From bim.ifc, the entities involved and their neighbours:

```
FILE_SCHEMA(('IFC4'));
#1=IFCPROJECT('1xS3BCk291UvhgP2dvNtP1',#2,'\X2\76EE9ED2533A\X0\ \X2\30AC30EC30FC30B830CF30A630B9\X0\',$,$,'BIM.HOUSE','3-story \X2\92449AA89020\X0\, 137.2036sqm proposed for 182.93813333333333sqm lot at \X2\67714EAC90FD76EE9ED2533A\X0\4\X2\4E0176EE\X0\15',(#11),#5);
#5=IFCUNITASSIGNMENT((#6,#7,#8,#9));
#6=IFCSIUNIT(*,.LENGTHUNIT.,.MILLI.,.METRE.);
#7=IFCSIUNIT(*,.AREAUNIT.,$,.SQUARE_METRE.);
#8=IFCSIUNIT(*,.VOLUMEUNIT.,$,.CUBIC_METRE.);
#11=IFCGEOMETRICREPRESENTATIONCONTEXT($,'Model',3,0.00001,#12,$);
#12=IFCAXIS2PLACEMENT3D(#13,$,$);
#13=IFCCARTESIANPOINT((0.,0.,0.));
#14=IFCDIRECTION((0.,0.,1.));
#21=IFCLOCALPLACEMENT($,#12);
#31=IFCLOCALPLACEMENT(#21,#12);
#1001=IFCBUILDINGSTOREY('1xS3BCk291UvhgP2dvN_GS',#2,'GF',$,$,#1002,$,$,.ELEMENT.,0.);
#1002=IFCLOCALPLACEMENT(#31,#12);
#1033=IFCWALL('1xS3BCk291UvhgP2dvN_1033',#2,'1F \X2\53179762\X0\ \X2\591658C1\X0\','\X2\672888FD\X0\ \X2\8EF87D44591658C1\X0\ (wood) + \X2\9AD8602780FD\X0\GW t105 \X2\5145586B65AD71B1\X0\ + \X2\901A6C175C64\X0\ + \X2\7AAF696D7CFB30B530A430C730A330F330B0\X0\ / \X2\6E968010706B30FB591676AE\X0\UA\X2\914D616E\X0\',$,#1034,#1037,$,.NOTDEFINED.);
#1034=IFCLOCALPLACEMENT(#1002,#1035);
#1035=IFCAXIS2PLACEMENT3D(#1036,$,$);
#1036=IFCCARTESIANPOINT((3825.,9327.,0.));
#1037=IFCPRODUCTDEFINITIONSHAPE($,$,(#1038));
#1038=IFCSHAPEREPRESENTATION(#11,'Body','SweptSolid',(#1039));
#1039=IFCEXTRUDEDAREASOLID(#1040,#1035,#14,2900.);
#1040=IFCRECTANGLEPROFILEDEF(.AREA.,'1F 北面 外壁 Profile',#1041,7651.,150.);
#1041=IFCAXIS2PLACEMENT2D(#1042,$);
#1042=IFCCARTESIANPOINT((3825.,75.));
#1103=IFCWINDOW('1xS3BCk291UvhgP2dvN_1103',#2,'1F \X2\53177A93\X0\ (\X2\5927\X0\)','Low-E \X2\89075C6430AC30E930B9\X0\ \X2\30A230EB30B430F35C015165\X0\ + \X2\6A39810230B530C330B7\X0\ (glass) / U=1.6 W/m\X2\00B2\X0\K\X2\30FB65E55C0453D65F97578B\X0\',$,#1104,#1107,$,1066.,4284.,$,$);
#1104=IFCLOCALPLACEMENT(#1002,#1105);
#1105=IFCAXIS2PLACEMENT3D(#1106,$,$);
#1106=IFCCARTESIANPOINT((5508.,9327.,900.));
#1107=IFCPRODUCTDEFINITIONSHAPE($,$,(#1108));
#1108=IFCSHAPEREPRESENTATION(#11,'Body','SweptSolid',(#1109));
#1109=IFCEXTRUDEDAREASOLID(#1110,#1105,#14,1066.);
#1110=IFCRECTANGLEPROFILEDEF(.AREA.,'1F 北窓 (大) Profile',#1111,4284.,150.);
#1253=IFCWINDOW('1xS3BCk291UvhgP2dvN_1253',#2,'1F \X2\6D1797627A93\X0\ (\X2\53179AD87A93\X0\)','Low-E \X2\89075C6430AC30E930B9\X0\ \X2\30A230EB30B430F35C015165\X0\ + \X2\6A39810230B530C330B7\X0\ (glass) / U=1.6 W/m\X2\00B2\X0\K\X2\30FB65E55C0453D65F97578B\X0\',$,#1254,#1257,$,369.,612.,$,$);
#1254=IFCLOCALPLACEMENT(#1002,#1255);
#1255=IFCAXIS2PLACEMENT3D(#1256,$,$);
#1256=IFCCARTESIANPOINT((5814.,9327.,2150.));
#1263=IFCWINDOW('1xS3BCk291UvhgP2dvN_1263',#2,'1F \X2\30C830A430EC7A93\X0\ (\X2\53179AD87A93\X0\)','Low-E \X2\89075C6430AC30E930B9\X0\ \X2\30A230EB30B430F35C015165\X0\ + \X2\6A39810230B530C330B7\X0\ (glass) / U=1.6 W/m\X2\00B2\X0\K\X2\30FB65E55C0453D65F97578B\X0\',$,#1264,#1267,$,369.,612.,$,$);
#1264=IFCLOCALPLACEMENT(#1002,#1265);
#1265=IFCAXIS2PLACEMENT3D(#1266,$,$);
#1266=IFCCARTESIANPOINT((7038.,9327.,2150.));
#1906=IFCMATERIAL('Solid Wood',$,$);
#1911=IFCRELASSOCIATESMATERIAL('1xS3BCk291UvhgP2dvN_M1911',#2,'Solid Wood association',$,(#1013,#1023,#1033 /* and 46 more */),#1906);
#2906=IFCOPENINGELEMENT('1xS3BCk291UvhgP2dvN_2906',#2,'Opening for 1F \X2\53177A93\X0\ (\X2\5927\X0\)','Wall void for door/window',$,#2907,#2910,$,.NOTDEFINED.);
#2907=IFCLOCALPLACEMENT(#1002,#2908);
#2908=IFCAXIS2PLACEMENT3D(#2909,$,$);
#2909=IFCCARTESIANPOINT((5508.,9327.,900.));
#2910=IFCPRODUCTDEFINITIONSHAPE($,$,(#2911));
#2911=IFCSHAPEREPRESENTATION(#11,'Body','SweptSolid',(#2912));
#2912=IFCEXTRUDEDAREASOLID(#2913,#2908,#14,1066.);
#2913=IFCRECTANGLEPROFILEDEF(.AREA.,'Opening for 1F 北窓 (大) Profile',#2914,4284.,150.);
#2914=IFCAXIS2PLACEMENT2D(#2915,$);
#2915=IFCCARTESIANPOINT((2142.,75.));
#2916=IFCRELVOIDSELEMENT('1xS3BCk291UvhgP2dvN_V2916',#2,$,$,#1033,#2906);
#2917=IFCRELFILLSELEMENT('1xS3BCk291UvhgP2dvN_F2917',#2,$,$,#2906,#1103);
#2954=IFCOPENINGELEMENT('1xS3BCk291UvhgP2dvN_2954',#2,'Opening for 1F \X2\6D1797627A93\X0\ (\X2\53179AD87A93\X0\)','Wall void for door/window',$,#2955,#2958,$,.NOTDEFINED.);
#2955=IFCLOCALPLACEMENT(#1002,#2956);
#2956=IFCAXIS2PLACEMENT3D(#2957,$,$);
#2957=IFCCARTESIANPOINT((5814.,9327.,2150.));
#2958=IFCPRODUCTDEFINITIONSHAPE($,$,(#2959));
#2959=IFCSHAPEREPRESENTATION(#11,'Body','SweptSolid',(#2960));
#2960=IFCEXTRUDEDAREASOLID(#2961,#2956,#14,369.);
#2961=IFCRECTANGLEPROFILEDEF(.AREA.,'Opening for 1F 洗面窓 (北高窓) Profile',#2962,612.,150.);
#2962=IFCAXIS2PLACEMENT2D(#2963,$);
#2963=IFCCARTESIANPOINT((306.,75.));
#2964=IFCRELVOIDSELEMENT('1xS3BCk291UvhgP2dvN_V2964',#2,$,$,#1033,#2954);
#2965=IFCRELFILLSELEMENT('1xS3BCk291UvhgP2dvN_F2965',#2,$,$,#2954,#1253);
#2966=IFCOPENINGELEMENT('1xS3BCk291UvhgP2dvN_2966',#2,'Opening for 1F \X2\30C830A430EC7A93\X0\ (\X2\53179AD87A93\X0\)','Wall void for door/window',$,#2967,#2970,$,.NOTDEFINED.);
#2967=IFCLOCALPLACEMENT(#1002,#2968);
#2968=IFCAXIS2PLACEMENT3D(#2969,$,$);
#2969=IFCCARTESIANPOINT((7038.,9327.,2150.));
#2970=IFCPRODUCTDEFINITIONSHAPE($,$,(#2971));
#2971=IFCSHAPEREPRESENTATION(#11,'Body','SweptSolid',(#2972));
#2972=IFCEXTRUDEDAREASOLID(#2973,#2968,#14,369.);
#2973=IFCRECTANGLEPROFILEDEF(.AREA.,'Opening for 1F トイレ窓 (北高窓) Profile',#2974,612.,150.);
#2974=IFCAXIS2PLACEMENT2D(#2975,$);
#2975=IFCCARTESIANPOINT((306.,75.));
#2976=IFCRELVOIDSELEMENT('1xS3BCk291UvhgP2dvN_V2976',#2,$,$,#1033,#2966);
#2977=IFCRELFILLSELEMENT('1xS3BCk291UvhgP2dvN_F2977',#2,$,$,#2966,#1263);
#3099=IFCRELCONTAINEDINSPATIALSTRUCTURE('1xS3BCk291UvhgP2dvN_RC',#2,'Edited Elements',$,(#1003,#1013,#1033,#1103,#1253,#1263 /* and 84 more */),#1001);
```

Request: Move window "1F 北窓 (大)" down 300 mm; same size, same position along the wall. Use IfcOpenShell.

```python
import numpy as np
import ifcopenshell
import ifcopenshell.api.geometry
import ifcopenshell.util.placement
import ifcopenshell.util.unit

model = ifcopenshell.open("bim.ifc")
unit_scale = ifcopenshell.util.unit.calculate_unit_scale(model)

window = model.by_guid("1xS3BCk291UvhgP2dvN_1103")
opening = window.FillsVoids[0].RelatingOpeningElement
dz = -0.3 / unit_scale

shift = np.array([0.0, 0.0, dz])
# The window is not placed relative to its opening, so move both.
for product in (opening, window):
    matrix = ifcopenshell.util.placement.get_local_placement(product.ObjectPlacement)
    matrix[:3, 3] += shift
    ifcopenshell.api.geometry.edit_object_placement(model, product=product, matrix=matrix, is_si=False)

print(f"moved by {dz * unit_scale:+.3f} m")

model.write("bim_updated.ifc")
```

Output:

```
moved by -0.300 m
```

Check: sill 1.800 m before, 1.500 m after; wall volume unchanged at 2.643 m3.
